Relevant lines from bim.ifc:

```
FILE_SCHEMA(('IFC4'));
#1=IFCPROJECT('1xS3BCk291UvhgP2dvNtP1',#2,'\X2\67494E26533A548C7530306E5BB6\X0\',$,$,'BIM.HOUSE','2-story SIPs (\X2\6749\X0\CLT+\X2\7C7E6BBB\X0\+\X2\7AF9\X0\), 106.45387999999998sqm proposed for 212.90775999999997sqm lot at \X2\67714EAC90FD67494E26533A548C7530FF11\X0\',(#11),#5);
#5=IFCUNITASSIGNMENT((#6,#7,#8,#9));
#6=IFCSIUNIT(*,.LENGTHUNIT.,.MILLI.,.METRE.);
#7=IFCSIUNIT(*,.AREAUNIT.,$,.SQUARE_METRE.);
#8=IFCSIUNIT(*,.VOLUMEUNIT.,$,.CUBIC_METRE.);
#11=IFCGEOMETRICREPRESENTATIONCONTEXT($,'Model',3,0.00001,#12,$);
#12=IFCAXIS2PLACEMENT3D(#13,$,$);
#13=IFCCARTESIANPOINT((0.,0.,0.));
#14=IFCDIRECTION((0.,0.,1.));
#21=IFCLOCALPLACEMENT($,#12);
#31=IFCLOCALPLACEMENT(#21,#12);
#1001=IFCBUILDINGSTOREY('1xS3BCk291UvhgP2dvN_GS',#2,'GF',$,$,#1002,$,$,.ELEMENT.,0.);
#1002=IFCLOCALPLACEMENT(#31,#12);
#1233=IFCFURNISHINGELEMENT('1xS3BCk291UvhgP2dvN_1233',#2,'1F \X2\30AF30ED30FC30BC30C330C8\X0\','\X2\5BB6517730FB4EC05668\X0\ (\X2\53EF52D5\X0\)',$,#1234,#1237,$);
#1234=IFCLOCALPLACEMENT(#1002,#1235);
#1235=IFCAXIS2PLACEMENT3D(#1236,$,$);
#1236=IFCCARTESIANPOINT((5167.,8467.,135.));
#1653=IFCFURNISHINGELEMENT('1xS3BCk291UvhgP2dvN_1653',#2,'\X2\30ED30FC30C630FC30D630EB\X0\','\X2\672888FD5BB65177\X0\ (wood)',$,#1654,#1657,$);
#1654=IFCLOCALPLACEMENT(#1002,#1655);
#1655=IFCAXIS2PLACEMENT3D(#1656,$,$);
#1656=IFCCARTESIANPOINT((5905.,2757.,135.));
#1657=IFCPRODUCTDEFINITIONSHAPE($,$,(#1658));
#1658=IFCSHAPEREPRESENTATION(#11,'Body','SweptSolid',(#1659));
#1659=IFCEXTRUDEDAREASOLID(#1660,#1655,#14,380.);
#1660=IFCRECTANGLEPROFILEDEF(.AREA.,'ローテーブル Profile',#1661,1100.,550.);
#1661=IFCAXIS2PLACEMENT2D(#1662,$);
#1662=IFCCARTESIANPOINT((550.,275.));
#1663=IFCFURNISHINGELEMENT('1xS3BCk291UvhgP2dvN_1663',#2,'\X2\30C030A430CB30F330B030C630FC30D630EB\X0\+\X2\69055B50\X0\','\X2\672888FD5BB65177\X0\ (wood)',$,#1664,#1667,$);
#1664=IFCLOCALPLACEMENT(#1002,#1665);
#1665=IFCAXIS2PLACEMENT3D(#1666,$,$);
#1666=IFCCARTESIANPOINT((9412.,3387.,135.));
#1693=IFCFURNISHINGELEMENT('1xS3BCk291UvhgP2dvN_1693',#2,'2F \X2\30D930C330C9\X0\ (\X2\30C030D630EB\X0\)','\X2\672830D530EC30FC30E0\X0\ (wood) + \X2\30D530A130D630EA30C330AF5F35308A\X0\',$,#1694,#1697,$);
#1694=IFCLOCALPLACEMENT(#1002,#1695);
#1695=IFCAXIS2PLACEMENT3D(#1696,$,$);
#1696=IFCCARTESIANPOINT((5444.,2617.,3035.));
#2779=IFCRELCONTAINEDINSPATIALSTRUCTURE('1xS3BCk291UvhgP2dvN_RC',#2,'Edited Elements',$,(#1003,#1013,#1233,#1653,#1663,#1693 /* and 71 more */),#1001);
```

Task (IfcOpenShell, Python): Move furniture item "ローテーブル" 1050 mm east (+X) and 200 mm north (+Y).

```python
import ifcopenshell
import ifcopenshell.api.geometry
import ifcopenshell.util.placement
import ifcopenshell.util.unit

model = ifcopenshell.open("bim.ifc")
unit_scale = ifcopenshell.util.unit.calculate_unit_scale(model)

item = model.by_guid("1xS3BCk291UvhgP2dvN_1653")
matrix = ifcopenshell.util.placement.get_local_placement(item.ObjectPlacement)
matrix[0, 3] += 1.05 / unit_scale
matrix[1, 3] += 0.2 / unit_scale
ifcopenshell.api.geometry.edit_object_placement(model, product=item, matrix=matrix, is_si=False)

print(ifcopenshell.util.placement.get_local_placement(item.ObjectPlacement).round(3) + 0.0)

model.write("bim_v2.ifc")
```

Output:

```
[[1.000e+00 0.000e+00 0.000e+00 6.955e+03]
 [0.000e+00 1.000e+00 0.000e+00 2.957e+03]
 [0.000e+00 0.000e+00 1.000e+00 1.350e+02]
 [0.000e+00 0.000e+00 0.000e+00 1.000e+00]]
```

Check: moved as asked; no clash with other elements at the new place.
